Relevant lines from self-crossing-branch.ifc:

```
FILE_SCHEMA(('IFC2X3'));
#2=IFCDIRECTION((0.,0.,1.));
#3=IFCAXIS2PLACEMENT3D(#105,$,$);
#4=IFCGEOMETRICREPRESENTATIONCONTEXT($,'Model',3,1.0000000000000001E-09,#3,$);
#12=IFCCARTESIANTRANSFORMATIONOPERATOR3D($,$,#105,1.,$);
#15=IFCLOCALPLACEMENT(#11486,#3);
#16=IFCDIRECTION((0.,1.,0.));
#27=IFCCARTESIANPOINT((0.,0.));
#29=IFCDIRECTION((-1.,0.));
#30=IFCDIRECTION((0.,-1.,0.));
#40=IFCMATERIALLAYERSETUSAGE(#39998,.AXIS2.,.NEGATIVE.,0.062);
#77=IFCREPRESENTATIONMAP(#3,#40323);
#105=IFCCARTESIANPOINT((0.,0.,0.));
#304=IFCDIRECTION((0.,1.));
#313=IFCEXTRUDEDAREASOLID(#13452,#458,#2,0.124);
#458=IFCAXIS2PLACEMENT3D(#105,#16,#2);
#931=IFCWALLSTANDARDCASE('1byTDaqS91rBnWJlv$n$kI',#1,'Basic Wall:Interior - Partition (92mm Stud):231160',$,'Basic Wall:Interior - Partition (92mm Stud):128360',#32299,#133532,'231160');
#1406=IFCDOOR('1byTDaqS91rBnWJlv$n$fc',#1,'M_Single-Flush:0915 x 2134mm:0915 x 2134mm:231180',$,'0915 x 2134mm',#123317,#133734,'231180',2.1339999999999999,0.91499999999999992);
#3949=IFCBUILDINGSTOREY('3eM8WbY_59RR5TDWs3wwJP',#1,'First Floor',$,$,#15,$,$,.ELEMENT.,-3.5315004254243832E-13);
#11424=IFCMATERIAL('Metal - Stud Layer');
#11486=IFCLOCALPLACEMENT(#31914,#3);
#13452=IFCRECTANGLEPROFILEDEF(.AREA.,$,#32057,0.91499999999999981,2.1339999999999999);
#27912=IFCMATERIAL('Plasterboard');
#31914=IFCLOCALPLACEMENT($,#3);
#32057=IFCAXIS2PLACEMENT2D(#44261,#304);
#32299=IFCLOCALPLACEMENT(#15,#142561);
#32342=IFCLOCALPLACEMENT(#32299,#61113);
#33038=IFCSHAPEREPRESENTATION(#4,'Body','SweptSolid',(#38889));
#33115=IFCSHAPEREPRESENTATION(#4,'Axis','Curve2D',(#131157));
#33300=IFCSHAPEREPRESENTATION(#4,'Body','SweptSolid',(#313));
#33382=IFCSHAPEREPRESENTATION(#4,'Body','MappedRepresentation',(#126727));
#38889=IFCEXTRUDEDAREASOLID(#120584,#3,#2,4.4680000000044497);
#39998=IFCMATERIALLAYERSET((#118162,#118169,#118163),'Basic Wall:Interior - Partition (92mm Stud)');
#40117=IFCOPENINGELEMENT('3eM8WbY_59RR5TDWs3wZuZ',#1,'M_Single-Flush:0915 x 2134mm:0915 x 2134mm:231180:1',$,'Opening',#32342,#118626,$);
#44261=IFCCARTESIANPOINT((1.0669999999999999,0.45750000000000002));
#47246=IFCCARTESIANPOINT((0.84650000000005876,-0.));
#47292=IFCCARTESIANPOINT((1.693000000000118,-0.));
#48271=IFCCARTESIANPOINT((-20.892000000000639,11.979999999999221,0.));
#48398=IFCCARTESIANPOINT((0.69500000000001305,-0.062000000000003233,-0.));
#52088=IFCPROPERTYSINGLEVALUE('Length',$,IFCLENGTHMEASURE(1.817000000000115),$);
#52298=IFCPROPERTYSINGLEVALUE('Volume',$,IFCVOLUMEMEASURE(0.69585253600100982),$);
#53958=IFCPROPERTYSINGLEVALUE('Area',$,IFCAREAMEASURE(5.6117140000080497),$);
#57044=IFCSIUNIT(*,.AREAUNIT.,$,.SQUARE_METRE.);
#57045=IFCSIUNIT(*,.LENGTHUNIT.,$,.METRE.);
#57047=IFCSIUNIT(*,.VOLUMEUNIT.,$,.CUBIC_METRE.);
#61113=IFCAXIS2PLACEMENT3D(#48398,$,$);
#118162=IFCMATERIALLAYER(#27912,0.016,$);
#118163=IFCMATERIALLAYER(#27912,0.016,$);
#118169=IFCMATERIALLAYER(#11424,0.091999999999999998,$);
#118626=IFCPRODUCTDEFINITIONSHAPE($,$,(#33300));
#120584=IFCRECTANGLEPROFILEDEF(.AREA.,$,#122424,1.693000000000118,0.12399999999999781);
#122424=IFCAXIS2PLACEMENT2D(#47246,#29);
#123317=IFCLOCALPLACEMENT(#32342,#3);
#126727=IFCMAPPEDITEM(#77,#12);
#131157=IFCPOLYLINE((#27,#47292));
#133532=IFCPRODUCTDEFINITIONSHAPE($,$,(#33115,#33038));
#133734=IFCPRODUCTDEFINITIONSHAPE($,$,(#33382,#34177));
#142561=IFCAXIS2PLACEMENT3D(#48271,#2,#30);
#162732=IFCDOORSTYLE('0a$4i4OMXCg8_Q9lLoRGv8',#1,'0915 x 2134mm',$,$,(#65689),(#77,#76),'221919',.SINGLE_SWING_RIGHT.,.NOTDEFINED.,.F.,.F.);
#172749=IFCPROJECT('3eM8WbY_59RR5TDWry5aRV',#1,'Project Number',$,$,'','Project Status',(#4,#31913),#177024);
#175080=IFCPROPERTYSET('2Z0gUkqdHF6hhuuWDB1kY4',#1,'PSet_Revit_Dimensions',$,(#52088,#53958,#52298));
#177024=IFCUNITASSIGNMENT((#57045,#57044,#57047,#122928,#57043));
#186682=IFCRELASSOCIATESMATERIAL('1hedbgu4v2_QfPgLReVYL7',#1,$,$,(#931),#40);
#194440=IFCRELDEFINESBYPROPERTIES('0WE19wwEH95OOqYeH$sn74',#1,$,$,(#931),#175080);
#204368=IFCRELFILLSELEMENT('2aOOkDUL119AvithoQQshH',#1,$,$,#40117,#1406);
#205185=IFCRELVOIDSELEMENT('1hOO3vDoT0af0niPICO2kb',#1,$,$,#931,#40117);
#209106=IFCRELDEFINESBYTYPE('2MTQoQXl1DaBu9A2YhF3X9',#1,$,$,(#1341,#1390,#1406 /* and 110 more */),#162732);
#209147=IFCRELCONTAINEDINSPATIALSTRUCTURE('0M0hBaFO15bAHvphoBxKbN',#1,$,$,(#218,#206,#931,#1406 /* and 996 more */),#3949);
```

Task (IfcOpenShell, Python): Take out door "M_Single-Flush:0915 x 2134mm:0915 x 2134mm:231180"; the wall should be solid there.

```python
import ifcopenshell
import ifcopenshell.api.feature
import ifcopenshell.api.pset
import ifcopenshell.api.root
import ifcopenshell.geom
import ifcopenshell.util.element
import ifcopenshell.util.shape
import ifcopenshell.util.unit

model = ifcopenshell.open("self-crossing-branch.ifc")
area_scale = ifcopenshell.util.unit.calculate_unit_scale(model, "AREAUNIT")
volume_scale = ifcopenshell.util.unit.calculate_unit_scale(model, "VOLUMEUNIT")
settings = ifcopenshell.geom.settings()


def volume(element):
    """Net volume in cubic metres, openings subtracted."""
    shape = ifcopenshell.geom.create_shape(settings, element)
    return ifcopenshell.util.shape.get_volume(shape.geometry)


door = model.by_guid("1byTDaqS91rBnWJlv$n$fc")
opening = door.FillsVoids[0].RelatingOpeningElement
wall = opening.VoidsElements[0].RelatingBuildingElement
before = volume(wall)

ifcopenshell.api.root.remove_product(model, product=door)
ifcopenshell.api.feature.remove_feature(model, feature=opening)

after = volume(wall)
thickness = 0.124  # wall thickness in metres

# Update the wall's stored quantities.
pset = model.by_id(ifcopenshell.util.element.get_pset(wall, "PSet_Revit_Dimensions", should_inherit=False)["id"])
ifcopenshell.api.pset.edit_pset(model, pset=pset, properties={
    "Area": model.create_entity("IfcAreaMeasure", after / thickness / area_scale),
    "Volume": model.create_entity("IfcVolumeMeasure", after / volume_scale),
})

print(f"wall volume {before:.3f} -> {after:.3f} m3")

model.write("self-crossing-branch_rev.ifc")
```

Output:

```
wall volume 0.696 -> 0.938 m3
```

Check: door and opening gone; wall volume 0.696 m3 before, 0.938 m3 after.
